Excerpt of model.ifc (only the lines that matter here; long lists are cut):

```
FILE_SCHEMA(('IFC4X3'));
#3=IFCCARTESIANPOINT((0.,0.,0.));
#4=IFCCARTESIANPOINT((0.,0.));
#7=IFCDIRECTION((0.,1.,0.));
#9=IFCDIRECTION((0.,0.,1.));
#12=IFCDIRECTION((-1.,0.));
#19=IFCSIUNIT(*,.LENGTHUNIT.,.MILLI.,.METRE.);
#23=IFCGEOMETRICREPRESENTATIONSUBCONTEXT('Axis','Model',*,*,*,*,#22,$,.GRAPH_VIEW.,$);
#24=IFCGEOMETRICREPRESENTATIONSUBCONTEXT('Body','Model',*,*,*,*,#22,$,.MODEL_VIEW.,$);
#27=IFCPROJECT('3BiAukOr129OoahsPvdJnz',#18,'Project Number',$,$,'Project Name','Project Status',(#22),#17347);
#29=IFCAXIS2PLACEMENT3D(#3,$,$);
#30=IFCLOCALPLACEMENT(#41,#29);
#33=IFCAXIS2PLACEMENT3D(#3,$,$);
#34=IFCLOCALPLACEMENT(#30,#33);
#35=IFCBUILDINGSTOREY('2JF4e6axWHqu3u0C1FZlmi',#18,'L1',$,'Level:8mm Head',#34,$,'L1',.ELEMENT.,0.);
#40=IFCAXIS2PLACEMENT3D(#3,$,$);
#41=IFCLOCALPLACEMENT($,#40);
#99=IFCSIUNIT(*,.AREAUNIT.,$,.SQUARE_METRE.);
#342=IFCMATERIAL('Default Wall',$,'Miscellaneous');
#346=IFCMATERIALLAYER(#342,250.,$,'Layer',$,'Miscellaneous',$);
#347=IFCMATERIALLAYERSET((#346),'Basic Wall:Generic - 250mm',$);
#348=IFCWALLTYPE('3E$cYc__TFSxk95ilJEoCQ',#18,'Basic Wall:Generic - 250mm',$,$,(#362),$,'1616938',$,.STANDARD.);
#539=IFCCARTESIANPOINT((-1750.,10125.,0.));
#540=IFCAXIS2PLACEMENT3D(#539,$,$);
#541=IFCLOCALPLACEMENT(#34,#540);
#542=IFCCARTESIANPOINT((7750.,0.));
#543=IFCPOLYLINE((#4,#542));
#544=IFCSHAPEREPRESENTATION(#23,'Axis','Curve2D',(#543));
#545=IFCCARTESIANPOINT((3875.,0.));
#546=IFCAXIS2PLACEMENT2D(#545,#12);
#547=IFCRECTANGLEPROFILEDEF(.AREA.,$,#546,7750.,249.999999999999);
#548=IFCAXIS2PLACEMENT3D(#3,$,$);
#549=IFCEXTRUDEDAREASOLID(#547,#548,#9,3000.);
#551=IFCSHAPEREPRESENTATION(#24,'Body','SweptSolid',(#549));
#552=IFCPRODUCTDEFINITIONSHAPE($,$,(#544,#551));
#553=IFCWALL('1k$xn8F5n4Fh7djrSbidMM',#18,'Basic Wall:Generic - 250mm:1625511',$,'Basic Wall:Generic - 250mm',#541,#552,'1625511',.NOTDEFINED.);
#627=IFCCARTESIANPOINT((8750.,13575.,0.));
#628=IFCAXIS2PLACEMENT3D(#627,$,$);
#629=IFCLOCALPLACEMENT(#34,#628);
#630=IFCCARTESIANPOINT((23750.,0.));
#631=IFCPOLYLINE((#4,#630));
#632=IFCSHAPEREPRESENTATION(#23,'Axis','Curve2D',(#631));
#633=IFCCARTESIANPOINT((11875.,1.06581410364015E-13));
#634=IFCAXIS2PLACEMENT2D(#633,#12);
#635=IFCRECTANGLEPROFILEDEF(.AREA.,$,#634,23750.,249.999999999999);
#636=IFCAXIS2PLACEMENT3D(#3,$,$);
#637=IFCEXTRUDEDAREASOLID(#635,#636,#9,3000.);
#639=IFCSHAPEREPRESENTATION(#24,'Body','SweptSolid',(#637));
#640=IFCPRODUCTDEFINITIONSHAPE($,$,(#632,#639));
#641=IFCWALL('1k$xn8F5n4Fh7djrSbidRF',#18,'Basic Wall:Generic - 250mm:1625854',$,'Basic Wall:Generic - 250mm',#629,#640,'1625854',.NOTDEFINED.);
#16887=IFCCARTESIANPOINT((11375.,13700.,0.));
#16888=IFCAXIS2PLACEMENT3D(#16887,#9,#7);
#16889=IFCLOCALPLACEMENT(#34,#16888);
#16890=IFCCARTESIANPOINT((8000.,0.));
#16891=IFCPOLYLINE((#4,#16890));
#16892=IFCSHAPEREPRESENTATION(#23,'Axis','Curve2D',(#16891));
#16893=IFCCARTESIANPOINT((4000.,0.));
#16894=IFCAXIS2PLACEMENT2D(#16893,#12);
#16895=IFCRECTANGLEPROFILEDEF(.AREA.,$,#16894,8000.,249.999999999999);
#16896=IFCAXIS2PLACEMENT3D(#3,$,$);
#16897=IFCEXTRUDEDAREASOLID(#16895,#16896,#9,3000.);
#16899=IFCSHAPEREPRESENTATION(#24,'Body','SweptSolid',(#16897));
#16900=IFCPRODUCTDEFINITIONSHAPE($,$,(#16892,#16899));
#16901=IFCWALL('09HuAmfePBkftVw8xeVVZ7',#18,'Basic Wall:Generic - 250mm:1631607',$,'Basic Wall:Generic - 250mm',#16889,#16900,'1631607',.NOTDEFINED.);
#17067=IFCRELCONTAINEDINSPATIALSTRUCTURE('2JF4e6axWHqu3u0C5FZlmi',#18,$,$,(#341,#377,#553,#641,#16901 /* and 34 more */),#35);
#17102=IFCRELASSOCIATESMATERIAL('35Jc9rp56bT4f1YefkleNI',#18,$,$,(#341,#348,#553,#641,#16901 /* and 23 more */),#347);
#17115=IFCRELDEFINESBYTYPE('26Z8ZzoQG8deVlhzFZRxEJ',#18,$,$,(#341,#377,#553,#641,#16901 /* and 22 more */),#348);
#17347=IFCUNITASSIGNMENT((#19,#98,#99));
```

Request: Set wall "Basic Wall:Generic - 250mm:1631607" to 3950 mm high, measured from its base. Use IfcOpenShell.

```python
import ifcopenshell
import ifcopenshell.geom
import ifcopenshell.util.representation
import ifcopenshell.util.shape

model = ifcopenshell.open("model.ifc")
settings = ifcopenshell.geom.settings()


def volume(element):
    """Net volume in cubic metres, openings subtracted."""
    shape = ifcopenshell.geom.create_shape(settings, element)
    return ifcopenshell.util.shape.get_volume(shape.geometry)


wall = model.by_guid("09HuAmfePBkftVw8xeVVZ7")
before = volume(wall)

body = ifcopenshell.util.representation.get_representation(wall, "Model", "Body")
solid = body.Items[0]
old_height = solid.Depth
solid.Depth = 3950.0
after = volume(wall)

print(f"height {old_height:g} -> {solid.Depth:g}, volume {before:.3f} -> {after:.3f} m3")

model.write("model-out.ifc")
```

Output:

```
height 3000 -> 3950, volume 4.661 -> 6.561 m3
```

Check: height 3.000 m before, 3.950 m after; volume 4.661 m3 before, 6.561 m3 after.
